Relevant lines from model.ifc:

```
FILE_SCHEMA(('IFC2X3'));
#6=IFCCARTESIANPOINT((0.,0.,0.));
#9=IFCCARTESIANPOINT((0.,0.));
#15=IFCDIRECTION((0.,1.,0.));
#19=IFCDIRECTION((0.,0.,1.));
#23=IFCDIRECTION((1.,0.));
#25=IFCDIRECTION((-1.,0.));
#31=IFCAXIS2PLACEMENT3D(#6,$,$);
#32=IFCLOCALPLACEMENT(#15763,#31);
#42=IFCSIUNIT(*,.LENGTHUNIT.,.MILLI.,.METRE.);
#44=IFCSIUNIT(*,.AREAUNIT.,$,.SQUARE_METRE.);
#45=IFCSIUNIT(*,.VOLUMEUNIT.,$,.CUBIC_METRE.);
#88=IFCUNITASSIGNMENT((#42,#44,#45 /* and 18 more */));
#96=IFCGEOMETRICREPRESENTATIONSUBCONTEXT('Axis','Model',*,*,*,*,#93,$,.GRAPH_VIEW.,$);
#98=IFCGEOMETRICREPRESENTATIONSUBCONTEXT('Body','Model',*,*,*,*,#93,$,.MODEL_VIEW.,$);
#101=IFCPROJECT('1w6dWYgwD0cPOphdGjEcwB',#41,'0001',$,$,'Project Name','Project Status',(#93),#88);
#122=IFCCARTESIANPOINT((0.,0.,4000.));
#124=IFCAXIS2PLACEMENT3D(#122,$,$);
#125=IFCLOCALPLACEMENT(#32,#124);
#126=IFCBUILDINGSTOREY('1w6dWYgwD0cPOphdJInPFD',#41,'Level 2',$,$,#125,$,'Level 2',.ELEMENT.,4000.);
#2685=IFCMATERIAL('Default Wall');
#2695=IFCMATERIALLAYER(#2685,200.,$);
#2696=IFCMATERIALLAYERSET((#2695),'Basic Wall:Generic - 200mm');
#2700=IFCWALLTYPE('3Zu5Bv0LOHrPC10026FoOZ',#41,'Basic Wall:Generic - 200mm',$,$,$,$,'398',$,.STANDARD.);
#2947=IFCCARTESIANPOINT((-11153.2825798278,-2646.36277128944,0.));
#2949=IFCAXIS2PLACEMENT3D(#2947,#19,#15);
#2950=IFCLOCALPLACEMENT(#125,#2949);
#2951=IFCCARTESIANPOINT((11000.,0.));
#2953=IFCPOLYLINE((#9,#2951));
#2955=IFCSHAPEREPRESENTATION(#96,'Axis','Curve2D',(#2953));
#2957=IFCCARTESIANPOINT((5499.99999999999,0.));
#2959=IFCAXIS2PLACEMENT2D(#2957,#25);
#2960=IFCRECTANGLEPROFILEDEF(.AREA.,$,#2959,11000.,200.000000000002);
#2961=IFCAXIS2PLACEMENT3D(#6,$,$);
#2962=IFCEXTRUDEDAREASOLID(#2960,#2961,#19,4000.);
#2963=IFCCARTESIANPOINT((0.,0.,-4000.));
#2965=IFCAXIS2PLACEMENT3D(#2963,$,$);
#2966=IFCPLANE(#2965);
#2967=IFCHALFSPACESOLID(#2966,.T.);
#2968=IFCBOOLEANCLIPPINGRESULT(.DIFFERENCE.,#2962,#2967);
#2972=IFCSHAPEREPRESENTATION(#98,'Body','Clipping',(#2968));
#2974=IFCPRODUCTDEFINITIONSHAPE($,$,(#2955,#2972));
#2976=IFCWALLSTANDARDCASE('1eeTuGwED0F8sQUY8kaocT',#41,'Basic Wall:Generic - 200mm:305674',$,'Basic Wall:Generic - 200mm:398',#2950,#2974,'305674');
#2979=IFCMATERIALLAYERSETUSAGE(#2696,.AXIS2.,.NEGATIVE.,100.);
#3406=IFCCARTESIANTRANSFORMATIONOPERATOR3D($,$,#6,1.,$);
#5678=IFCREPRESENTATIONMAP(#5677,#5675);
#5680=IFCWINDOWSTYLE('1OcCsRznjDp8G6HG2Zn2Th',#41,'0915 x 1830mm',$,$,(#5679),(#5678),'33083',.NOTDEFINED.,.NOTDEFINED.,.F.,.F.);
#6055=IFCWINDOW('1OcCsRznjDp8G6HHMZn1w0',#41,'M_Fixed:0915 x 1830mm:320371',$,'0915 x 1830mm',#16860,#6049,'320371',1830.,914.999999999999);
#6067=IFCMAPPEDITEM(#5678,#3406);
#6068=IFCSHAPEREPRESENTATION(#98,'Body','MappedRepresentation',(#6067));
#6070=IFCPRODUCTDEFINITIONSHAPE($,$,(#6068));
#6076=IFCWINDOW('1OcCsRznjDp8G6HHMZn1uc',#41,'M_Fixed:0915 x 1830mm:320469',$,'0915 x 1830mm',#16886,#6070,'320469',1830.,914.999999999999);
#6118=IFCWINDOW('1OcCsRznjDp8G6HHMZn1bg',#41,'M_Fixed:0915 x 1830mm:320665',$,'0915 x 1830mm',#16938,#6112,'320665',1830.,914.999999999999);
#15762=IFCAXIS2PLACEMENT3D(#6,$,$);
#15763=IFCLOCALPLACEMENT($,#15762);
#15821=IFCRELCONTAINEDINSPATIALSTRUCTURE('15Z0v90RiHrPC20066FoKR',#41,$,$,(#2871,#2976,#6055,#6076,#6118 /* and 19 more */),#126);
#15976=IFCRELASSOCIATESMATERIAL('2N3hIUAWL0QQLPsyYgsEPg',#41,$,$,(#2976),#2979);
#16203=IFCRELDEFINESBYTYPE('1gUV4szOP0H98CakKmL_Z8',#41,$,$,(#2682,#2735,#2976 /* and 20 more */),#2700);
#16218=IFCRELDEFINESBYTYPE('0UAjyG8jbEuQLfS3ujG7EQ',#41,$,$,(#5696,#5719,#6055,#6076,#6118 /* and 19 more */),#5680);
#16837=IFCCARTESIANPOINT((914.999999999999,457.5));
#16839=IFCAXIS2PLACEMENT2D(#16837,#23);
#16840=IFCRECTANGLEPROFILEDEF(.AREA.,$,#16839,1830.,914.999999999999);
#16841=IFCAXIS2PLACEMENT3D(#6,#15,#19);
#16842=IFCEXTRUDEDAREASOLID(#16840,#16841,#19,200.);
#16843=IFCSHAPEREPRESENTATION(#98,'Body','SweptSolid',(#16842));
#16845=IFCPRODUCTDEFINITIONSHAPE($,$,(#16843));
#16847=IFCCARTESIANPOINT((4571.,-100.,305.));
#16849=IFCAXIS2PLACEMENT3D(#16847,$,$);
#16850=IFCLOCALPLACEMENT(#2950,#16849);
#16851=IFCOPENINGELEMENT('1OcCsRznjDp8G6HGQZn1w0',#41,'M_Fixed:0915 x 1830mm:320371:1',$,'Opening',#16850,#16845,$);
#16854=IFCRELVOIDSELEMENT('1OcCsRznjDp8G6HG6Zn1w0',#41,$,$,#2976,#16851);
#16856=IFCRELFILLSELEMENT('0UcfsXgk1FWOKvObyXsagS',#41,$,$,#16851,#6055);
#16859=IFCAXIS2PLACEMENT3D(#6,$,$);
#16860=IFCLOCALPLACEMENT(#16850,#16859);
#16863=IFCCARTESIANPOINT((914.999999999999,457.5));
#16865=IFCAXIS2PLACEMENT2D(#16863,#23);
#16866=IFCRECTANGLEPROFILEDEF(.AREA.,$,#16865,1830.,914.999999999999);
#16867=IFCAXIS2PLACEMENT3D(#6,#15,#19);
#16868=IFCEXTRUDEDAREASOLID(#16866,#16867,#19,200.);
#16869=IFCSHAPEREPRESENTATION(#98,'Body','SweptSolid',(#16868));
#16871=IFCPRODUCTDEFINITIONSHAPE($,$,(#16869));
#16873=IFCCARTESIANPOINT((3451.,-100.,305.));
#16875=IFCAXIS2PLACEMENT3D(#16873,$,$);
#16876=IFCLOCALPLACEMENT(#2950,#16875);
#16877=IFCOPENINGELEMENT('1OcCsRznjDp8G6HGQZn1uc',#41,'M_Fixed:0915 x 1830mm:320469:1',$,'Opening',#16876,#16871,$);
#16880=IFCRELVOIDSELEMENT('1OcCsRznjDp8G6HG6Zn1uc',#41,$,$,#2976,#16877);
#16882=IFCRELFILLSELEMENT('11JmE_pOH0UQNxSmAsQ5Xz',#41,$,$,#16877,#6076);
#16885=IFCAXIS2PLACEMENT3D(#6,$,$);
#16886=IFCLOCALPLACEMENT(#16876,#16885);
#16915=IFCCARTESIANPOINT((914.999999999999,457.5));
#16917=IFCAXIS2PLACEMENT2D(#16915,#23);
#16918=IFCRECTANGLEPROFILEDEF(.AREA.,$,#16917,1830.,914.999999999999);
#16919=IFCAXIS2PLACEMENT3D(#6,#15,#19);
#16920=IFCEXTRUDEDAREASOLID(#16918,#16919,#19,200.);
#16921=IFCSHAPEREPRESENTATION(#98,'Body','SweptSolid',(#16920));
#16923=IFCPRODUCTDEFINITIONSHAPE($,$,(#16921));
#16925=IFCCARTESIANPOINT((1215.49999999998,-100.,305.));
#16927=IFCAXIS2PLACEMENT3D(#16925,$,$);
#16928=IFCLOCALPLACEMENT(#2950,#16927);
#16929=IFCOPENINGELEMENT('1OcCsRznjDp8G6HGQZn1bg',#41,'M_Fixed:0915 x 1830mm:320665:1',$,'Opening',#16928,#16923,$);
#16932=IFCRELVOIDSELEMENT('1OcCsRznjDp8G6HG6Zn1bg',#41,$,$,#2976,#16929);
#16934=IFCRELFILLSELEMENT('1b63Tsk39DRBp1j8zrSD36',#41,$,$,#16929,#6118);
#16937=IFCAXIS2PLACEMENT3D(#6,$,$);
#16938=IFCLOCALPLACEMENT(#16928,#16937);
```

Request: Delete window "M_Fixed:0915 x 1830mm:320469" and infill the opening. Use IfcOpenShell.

```python
import ifcopenshell
import ifcopenshell.api.feature
import ifcopenshell.api.root
import ifcopenshell.geom
import ifcopenshell.util.shape

model = ifcopenshell.open("model.ifc")
settings = ifcopenshell.geom.settings()


def volume(element):
    """Net volume in cubic metres, openings subtracted."""
    shape = ifcopenshell.geom.create_shape(settings, element)
    return ifcopenshell.util.shape.get_volume(shape.geometry)


window = model.by_id(6076)
opening = window.FillsVoids[0].RelatingOpeningElement
wall = opening.VoidsElements[0].RelatingBuildingElement
before = volume(wall)

ifcopenshell.api.root.remove_product(model, product=window)
ifcopenshell.api.feature.remove_feature(model, feature=opening)

after = volume(wall)

print(f"wall volume {before:.3f} -> {after:.3f} m3")

model.write("model_v2.ifc")
```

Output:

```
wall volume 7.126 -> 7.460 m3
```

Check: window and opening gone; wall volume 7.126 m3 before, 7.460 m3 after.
